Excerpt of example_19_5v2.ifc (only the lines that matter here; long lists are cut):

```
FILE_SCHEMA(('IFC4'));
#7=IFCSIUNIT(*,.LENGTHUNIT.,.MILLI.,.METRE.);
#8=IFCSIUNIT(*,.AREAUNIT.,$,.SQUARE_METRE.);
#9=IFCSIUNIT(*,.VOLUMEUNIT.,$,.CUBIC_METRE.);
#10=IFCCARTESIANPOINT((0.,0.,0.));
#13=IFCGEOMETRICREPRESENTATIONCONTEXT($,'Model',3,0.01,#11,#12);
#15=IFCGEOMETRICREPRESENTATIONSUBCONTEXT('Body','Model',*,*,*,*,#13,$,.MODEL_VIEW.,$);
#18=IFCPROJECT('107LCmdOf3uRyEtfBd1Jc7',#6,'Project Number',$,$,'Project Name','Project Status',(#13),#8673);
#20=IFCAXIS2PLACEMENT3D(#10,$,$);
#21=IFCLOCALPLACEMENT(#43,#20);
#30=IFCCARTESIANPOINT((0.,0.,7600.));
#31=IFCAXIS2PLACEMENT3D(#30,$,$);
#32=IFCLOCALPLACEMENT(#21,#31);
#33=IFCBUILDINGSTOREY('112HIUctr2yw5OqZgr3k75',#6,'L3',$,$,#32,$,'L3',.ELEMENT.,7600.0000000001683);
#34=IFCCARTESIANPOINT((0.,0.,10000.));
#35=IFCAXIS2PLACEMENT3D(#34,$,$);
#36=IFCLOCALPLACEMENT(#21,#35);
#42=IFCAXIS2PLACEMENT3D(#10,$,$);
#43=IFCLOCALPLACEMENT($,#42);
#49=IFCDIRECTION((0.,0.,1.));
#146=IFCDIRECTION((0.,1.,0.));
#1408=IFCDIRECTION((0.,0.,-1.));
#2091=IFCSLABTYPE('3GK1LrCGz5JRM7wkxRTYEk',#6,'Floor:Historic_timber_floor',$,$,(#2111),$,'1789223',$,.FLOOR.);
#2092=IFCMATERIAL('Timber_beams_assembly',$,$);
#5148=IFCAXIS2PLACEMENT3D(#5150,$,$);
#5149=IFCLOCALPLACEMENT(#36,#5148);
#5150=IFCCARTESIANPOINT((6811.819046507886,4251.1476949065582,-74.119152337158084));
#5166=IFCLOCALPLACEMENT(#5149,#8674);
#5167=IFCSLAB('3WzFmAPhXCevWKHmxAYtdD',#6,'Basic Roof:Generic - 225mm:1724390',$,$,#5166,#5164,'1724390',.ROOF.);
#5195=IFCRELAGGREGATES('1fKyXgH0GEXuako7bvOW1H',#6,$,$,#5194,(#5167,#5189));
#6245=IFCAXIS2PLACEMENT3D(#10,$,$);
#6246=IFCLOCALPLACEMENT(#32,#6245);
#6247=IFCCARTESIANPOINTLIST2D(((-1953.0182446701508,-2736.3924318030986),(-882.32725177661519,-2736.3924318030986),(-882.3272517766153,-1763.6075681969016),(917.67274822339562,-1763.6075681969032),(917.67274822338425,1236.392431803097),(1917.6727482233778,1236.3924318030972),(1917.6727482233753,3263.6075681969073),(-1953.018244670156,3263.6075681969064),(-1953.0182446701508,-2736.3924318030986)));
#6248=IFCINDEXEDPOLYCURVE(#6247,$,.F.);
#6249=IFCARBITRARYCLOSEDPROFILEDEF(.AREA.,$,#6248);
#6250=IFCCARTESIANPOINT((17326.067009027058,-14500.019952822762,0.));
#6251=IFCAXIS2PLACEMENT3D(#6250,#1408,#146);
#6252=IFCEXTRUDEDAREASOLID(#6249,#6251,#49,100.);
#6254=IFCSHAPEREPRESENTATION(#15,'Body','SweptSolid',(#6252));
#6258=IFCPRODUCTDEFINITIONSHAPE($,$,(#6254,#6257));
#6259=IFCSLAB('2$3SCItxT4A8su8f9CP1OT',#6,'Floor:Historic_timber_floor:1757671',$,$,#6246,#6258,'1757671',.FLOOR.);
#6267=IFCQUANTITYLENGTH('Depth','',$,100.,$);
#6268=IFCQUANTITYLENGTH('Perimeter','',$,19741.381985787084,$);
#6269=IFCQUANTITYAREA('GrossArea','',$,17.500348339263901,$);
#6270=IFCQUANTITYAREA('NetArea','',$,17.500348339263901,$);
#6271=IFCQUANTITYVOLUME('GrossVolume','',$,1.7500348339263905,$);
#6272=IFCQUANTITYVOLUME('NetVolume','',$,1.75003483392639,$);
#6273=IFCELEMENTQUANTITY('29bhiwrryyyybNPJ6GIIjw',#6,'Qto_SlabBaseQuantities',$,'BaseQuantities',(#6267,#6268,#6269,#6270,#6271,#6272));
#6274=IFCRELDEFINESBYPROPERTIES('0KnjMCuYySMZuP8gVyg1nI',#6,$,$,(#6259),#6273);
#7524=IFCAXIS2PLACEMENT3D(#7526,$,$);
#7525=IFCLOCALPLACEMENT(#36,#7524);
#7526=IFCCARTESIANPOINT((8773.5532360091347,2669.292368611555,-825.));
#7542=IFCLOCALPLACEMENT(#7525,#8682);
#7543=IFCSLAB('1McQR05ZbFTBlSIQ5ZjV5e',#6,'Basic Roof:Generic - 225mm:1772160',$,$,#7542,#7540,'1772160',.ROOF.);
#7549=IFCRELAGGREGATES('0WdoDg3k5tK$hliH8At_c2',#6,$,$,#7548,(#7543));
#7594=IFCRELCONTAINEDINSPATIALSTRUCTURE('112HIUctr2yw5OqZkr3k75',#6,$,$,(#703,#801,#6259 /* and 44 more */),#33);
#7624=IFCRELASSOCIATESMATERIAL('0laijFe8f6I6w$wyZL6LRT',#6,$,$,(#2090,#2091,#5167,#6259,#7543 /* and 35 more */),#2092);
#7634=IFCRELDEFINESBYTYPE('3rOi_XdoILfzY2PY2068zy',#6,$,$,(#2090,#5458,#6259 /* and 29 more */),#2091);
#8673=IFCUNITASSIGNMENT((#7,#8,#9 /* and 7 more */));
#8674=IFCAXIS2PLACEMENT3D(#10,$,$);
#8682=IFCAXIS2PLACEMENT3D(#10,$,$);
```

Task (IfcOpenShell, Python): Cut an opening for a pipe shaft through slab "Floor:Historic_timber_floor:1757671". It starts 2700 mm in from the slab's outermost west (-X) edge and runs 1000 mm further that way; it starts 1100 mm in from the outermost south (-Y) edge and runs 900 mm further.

```python
import numpy as np
import ifcopenshell
import ifcopenshell.api.feature
import ifcopenshell.api.geometry
import ifcopenshell.api.pset
import ifcopenshell.api.root
import ifcopenshell.geom
import ifcopenshell.util.element
import ifcopenshell.util.placement
import ifcopenshell.util.representation
import ifcopenshell.util.shape
import ifcopenshell.util.unit

model = ifcopenshell.open("example_19_5v2.ifc")
unit_scale = ifcopenshell.util.unit.calculate_unit_scale(model)
area_scale = ifcopenshell.util.unit.calculate_unit_scale(model, "AREAUNIT")
volume_scale = ifcopenshell.util.unit.calculate_unit_scale(model, "VOLUMEUNIT")
settings = ifcopenshell.geom.settings()


def volume(element):
    """Net volume in cubic metres, openings subtracted."""
    shape = ifcopenshell.geom.create_shape(settings, element)
    return ifcopenshell.util.shape.get_volume(shape.geometry)


slab = model.by_id(6259)
before = volume(slab)

# Extent in the slab's own axes, in metres. The edges named are its -X and -Y sides.
slab_shape = ifcopenshell.geom.create_shape(settings, slab)
vertices = ifcopenshell.util.shape.get_vertices(slab_shape.geometry)
x_min, y_min, bottom = vertices.min(axis=0)
top = vertices[:, 2].max()

opening = ifcopenshell.api.root.create_entity(model, ifc_class="IfcOpeningElement", name="Pipe shaft opening", predefined_type="OPENING")
context = ifcopenshell.util.representation.get_context(model, "Model", "Body", "MODEL_VIEW")
width, depth = 1, 0.9
outline = [(0.0, 0.0), (width, 0.0), (width, depth), (0.0, depth), (0.0, 0.0)]
# Overshoot both faces by 50 mm so the cut is clean.
shape = ifcopenshell.api.geometry.add_slab_representation(
    model, context=context, depth=top - bottom + 0.1, polyline=outline
)
ifcopenshell.api.geometry.assign_representation(model, product=opening, representation=shape)

matrix = ifcopenshell.util.placement.get_local_placement(slab.ObjectPlacement)
matrix[:, 3] = matrix @ np.append(np.array([x_min + 2.7, y_min + 1.1, bottom - 0.05]) / unit_scale, 1.0)
ifcopenshell.api.geometry.edit_object_placement(model, product=opening, matrix=matrix, is_si=False)
ifcopenshell.api.feature.add_feature(model, feature=opening, element=slab)

after = volume(slab)

# Update the slab's stored quantities.
qto = model.by_id(ifcopenshell.util.element.get_pset(slab, "Qto_SlabBaseQuantities", should_inherit=False)["id"])
ifcopenshell.api.pset.edit_qto(model, qto=qto, properties={
    "NetArea": after / (top - bottom) / area_scale,
    "NetVolume": after / volume_scale,
})

print(f"slab volume {before:.3f} -> {after:.3f} m3")

model.write("example_19_5v2-out.ifc")
```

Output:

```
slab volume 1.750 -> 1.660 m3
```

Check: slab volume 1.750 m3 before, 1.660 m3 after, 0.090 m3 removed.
